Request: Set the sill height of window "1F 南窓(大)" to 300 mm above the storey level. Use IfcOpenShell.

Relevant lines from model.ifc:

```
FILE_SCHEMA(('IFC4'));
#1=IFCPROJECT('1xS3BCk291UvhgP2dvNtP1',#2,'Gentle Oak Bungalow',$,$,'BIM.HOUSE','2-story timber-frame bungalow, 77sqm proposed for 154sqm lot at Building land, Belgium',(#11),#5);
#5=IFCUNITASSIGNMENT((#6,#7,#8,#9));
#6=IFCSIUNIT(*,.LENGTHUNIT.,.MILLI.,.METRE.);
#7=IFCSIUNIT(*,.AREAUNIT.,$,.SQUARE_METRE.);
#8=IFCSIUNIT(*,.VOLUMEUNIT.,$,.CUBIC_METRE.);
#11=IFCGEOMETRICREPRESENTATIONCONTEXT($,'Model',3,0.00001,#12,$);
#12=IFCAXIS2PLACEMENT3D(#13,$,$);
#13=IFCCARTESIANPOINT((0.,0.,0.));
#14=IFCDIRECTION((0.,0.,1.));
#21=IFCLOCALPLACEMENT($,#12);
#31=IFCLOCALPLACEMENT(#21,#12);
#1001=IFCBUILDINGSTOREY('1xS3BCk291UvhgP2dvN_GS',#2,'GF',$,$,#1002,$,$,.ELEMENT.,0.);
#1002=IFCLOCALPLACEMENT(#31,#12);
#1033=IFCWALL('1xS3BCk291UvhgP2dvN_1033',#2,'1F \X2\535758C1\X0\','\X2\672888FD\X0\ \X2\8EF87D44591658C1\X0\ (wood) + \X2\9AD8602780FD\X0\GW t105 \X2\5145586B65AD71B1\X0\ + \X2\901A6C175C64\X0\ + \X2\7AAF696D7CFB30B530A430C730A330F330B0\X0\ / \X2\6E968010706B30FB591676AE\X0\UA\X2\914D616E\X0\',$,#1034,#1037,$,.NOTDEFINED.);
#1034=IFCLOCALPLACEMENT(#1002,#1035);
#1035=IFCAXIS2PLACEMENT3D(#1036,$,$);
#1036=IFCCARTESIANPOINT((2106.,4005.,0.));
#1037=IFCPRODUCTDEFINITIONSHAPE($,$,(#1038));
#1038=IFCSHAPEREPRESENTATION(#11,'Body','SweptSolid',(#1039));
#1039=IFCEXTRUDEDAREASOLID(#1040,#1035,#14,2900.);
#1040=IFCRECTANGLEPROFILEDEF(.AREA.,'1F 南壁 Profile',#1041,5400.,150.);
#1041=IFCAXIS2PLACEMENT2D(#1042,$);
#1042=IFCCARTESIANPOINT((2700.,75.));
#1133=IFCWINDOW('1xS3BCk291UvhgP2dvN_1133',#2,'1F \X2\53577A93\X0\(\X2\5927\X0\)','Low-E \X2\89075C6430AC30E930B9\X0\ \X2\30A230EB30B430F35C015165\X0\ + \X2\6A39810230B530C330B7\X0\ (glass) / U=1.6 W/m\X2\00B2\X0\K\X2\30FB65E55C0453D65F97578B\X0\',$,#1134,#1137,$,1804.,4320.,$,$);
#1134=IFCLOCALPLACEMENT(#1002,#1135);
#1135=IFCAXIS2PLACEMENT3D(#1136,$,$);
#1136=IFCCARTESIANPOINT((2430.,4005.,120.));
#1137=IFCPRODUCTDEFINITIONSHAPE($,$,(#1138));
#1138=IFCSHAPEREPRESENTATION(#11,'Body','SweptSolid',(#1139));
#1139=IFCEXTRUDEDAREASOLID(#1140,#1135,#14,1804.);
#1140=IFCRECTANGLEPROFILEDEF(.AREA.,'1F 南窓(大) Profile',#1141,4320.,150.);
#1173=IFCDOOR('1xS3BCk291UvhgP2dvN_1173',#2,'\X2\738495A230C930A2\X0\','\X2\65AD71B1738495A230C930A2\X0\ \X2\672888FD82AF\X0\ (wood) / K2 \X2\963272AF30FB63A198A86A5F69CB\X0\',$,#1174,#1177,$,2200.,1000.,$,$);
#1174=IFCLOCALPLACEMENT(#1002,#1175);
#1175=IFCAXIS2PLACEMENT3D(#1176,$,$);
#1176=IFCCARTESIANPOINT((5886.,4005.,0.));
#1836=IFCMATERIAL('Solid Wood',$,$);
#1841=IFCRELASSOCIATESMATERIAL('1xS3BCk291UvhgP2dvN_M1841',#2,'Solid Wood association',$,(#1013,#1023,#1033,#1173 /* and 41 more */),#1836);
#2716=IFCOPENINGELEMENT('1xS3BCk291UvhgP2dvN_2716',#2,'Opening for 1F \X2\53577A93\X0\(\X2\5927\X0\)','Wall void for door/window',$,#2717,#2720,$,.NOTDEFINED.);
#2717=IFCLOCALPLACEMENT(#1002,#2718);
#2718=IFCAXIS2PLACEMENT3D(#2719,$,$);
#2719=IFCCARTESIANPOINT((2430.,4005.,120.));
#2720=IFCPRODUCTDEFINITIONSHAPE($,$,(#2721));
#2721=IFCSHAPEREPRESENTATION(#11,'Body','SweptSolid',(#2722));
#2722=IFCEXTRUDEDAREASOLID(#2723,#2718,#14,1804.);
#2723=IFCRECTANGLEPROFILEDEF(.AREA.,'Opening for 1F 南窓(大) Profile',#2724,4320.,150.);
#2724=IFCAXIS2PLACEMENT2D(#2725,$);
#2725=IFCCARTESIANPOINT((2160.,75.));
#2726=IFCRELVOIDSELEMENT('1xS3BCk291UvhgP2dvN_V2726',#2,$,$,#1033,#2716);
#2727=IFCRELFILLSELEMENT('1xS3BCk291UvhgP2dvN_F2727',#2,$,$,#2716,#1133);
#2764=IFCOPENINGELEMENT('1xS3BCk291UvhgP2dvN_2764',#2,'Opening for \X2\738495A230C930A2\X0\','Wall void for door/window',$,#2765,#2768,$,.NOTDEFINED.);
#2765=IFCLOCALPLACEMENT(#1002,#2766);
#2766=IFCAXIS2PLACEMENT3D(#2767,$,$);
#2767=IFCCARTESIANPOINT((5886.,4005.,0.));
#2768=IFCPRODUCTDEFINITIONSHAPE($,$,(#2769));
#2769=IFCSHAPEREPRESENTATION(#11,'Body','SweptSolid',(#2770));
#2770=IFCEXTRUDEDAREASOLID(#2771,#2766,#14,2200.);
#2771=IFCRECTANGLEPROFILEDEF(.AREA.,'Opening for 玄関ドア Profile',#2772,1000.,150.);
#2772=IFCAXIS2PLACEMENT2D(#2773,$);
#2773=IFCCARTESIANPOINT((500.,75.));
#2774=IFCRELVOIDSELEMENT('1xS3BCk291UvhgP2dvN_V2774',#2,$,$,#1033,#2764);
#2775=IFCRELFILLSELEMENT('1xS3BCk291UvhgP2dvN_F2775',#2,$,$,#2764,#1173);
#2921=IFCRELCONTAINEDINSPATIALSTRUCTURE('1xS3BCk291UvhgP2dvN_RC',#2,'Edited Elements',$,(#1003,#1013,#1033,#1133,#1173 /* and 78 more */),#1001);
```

```python
import numpy as np
import ifcopenshell
import ifcopenshell.api.geometry
import ifcopenshell.geom
import ifcopenshell.util.element
import ifcopenshell.util.placement
import ifcopenshell.util.shape
import ifcopenshell.util.unit

model = ifcopenshell.open("model.ifc")
unit_scale = ifcopenshell.util.unit.calculate_unit_scale(model)

window = model.by_guid("1xS3BCk291UvhgP2dvN_1133")
opening = window.FillsVoids[0].RelatingOpeningElement
storey = ifcopenshell.util.element.get_container(window, ifc_class="IfcBuildingStorey")
level = ifcopenshell.util.placement.get_local_placement(storey.ObjectPlacement)[2, 3]

# The opening's origin need not be at the sill, so measure its lowest point.
shape = ifcopenshell.geom.create_shape(ifcopenshell.geom.settings(), opening)
bottom = ifcopenshell.util.shape.get_shape_bottom_elevation(shape, shape.geometry) / unit_scale
dz = level + 300.0 - bottom

shift = np.array([0.0, 0.0, dz])
# The window is not placed relative to its opening, so move both.
for product in (opening, window):
    matrix = ifcopenshell.util.placement.get_local_placement(product.ObjectPlacement)
    matrix[:3, 3] += shift
    ifcopenshell.api.geometry.edit_object_placement(model, product=product, matrix=matrix, is_si=False)

print(f"moved by {dz * unit_scale:+.3f} m")

model.write("model_edited.ifc")
```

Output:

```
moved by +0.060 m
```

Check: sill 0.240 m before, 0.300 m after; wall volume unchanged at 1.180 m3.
